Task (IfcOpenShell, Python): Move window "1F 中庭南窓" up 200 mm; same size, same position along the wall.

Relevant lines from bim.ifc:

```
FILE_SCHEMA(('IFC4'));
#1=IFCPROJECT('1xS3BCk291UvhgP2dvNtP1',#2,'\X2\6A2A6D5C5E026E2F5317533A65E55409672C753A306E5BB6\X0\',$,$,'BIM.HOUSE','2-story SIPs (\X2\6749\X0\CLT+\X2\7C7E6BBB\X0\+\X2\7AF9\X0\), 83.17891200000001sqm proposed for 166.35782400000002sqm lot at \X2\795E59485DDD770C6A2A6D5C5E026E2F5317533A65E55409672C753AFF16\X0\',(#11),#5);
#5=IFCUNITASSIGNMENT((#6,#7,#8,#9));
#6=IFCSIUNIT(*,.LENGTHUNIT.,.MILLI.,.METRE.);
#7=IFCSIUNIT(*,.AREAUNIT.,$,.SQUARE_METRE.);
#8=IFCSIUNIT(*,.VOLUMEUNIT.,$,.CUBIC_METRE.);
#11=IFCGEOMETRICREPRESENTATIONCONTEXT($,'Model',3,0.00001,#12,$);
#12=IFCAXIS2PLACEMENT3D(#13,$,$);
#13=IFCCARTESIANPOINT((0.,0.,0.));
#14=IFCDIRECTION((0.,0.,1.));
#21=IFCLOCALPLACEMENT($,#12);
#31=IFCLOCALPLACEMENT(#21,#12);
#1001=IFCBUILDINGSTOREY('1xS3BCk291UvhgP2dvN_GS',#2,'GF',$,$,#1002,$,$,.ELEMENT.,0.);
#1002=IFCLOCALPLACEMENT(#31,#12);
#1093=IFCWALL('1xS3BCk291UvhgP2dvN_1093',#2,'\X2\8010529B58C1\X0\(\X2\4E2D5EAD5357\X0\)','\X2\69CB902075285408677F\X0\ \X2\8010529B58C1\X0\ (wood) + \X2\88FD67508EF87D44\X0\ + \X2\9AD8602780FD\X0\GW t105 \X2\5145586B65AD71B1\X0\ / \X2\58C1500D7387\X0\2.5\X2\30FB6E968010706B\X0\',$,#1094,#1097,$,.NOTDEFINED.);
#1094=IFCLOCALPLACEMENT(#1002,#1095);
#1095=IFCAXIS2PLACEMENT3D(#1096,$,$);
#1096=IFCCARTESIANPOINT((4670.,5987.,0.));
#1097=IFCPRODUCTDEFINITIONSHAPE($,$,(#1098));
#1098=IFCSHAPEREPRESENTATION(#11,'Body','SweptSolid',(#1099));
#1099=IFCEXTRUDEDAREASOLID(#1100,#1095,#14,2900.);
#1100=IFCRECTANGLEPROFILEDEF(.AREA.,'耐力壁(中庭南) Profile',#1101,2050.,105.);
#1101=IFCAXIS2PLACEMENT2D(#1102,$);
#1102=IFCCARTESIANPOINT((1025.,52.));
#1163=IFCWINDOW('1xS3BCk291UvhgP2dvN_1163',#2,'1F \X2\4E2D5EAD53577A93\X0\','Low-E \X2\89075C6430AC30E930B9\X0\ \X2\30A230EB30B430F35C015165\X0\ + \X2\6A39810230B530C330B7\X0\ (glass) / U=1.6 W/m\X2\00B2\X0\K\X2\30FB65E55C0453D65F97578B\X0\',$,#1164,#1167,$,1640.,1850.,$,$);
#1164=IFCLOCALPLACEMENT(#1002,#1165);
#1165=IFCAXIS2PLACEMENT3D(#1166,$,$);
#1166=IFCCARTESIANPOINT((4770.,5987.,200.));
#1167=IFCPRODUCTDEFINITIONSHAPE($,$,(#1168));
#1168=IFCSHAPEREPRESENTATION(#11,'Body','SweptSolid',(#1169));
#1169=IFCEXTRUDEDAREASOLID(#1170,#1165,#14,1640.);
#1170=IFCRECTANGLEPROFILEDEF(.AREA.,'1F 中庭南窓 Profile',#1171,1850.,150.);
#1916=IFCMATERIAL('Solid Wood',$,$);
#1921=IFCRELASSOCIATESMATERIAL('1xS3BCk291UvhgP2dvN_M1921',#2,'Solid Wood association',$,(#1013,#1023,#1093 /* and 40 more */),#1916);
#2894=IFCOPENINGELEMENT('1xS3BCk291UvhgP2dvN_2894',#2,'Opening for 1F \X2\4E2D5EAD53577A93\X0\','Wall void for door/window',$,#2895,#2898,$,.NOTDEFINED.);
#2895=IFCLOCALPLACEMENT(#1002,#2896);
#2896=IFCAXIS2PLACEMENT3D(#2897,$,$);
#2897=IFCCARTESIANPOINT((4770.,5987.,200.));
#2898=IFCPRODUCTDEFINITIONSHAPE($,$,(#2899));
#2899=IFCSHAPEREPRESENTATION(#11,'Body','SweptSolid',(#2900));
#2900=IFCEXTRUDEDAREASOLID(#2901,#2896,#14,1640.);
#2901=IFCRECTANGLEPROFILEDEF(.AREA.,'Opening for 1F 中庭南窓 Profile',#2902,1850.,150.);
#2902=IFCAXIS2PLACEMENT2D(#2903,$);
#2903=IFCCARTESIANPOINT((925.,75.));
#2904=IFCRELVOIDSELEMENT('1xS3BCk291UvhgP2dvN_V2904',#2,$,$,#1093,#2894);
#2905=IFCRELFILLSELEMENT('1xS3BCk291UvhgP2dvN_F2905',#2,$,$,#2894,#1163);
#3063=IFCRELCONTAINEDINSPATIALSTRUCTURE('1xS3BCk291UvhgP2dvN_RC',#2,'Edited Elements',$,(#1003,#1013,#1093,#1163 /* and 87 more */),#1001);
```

```python
import numpy as np
import ifcopenshell
import ifcopenshell.api.geometry
import ifcopenshell.util.placement
import ifcopenshell.util.unit

model = ifcopenshell.open("bim.ifc")
unit_scale = ifcopenshell.util.unit.calculate_unit_scale(model)

window = model.by_guid("1xS3BCk291UvhgP2dvN_1163")
opening = window.FillsVoids[0].RelatingOpeningElement
dz = 200.0

shift = np.array([0.0, 0.0, dz])
# The window is not placed relative to its opening, so move both.
for product in (opening, window):
    matrix = ifcopenshell.util.placement.get_local_placement(product.ObjectPlacement)
    matrix[:3, 3] += shift
    ifcopenshell.api.geometry.edit_object_placement(model, product=product, matrix=matrix, is_si=False)

print(f"moved by {dz * unit_scale:+.3f} m")

model.write("bim_rev.ifc")
```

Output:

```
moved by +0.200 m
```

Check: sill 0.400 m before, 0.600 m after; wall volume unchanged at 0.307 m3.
